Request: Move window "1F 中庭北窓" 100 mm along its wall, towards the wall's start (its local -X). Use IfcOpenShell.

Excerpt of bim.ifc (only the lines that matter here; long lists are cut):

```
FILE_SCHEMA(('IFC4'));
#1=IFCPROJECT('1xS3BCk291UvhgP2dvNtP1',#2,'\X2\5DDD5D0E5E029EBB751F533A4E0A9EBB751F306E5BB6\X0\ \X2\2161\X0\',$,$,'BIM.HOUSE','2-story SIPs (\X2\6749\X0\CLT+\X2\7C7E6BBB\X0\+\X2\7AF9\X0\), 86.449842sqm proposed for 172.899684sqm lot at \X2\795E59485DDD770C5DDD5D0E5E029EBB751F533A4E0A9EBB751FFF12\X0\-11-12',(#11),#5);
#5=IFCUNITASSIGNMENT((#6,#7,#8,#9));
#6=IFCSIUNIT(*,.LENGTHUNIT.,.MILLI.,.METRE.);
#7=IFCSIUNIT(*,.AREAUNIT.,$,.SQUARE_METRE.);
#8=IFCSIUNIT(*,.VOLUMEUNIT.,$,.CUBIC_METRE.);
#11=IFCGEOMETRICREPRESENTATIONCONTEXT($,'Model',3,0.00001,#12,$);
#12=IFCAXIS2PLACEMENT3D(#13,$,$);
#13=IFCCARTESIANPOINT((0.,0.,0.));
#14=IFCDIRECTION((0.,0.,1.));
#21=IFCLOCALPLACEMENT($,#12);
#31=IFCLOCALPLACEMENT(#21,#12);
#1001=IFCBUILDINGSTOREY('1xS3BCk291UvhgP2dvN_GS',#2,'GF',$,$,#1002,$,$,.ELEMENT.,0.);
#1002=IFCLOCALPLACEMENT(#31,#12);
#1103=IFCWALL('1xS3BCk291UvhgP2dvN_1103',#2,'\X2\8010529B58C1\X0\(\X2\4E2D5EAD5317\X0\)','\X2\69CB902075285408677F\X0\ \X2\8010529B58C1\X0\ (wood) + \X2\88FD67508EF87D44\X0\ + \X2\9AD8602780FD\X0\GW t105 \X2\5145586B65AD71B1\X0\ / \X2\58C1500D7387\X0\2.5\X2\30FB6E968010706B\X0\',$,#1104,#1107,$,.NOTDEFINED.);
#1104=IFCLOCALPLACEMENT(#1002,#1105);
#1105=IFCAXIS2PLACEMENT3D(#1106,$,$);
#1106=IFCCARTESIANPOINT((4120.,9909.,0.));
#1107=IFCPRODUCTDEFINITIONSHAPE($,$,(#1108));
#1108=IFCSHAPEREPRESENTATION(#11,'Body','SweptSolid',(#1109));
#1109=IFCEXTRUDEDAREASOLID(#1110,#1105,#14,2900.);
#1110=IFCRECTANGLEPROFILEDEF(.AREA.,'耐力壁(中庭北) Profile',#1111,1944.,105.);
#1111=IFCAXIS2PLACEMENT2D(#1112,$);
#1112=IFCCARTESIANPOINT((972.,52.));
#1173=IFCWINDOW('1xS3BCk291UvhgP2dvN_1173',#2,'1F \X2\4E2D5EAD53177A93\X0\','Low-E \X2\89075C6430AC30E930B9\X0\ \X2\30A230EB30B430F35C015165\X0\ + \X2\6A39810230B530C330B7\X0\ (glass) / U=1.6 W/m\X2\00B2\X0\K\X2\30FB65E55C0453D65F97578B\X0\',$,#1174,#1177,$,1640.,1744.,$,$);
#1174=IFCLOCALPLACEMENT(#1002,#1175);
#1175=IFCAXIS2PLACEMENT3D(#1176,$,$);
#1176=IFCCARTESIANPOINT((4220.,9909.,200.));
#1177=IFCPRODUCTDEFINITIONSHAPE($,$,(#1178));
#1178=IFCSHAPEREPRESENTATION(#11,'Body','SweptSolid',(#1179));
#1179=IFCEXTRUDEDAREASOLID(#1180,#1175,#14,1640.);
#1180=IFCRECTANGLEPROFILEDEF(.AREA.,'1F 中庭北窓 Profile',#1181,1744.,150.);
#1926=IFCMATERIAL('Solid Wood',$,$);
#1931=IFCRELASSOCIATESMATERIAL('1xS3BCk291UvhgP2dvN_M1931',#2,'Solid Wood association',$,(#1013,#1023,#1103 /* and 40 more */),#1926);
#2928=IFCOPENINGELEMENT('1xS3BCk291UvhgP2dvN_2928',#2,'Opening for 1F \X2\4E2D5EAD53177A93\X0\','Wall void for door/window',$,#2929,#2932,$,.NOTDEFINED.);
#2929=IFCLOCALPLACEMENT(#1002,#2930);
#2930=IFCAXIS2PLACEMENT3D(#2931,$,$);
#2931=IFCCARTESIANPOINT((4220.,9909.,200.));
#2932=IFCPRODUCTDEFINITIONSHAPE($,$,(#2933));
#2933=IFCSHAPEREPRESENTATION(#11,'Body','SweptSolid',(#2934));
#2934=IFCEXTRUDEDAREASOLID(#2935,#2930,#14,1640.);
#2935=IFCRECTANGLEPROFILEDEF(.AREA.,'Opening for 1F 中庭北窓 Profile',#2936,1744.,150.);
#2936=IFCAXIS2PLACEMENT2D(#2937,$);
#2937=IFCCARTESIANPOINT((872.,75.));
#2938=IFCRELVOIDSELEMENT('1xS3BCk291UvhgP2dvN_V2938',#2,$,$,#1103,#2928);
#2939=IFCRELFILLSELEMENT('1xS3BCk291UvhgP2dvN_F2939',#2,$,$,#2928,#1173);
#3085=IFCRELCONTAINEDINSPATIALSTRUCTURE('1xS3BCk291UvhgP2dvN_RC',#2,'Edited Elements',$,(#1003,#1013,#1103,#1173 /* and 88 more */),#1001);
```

```python
import ifcopenshell
import ifcopenshell.api.geometry
import ifcopenshell.util.placement
import ifcopenshell.util.unit

model = ifcopenshell.open("bim.ifc")
unit_scale = ifcopenshell.util.unit.calculate_unit_scale(model)

window = model.by_id(1173)
opening = window.FillsVoids[0].RelatingOpeningElement
wall = opening.VoidsElements[0].RelatingBuildingElement

wall_matrix = ifcopenshell.util.placement.get_local_placement(wall.ObjectPlacement)
shift = wall_matrix[:3, 0] * -0.1 / unit_scale
before = ifcopenshell.util.placement.get_local_placement(window.ObjectPlacement)[:3, 3].copy()

# The window is not placed relative to its opening, so move both.
for product in (opening, window):
    matrix = ifcopenshell.util.placement.get_local_placement(product.ObjectPlacement)
    matrix[:3, 3] += shift
    ifcopenshell.api.geometry.edit_object_placement(model, product=product, matrix=matrix, is_si=False)

after = ifcopenshell.util.placement.get_local_placement(window.ObjectPlacement)[:3, 3]
print("window moved by", (after - before).round(3) + 0.0)

model.write("bim_v2.ifc")
```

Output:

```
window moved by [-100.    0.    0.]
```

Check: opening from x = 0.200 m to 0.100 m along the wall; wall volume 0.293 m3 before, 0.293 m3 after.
